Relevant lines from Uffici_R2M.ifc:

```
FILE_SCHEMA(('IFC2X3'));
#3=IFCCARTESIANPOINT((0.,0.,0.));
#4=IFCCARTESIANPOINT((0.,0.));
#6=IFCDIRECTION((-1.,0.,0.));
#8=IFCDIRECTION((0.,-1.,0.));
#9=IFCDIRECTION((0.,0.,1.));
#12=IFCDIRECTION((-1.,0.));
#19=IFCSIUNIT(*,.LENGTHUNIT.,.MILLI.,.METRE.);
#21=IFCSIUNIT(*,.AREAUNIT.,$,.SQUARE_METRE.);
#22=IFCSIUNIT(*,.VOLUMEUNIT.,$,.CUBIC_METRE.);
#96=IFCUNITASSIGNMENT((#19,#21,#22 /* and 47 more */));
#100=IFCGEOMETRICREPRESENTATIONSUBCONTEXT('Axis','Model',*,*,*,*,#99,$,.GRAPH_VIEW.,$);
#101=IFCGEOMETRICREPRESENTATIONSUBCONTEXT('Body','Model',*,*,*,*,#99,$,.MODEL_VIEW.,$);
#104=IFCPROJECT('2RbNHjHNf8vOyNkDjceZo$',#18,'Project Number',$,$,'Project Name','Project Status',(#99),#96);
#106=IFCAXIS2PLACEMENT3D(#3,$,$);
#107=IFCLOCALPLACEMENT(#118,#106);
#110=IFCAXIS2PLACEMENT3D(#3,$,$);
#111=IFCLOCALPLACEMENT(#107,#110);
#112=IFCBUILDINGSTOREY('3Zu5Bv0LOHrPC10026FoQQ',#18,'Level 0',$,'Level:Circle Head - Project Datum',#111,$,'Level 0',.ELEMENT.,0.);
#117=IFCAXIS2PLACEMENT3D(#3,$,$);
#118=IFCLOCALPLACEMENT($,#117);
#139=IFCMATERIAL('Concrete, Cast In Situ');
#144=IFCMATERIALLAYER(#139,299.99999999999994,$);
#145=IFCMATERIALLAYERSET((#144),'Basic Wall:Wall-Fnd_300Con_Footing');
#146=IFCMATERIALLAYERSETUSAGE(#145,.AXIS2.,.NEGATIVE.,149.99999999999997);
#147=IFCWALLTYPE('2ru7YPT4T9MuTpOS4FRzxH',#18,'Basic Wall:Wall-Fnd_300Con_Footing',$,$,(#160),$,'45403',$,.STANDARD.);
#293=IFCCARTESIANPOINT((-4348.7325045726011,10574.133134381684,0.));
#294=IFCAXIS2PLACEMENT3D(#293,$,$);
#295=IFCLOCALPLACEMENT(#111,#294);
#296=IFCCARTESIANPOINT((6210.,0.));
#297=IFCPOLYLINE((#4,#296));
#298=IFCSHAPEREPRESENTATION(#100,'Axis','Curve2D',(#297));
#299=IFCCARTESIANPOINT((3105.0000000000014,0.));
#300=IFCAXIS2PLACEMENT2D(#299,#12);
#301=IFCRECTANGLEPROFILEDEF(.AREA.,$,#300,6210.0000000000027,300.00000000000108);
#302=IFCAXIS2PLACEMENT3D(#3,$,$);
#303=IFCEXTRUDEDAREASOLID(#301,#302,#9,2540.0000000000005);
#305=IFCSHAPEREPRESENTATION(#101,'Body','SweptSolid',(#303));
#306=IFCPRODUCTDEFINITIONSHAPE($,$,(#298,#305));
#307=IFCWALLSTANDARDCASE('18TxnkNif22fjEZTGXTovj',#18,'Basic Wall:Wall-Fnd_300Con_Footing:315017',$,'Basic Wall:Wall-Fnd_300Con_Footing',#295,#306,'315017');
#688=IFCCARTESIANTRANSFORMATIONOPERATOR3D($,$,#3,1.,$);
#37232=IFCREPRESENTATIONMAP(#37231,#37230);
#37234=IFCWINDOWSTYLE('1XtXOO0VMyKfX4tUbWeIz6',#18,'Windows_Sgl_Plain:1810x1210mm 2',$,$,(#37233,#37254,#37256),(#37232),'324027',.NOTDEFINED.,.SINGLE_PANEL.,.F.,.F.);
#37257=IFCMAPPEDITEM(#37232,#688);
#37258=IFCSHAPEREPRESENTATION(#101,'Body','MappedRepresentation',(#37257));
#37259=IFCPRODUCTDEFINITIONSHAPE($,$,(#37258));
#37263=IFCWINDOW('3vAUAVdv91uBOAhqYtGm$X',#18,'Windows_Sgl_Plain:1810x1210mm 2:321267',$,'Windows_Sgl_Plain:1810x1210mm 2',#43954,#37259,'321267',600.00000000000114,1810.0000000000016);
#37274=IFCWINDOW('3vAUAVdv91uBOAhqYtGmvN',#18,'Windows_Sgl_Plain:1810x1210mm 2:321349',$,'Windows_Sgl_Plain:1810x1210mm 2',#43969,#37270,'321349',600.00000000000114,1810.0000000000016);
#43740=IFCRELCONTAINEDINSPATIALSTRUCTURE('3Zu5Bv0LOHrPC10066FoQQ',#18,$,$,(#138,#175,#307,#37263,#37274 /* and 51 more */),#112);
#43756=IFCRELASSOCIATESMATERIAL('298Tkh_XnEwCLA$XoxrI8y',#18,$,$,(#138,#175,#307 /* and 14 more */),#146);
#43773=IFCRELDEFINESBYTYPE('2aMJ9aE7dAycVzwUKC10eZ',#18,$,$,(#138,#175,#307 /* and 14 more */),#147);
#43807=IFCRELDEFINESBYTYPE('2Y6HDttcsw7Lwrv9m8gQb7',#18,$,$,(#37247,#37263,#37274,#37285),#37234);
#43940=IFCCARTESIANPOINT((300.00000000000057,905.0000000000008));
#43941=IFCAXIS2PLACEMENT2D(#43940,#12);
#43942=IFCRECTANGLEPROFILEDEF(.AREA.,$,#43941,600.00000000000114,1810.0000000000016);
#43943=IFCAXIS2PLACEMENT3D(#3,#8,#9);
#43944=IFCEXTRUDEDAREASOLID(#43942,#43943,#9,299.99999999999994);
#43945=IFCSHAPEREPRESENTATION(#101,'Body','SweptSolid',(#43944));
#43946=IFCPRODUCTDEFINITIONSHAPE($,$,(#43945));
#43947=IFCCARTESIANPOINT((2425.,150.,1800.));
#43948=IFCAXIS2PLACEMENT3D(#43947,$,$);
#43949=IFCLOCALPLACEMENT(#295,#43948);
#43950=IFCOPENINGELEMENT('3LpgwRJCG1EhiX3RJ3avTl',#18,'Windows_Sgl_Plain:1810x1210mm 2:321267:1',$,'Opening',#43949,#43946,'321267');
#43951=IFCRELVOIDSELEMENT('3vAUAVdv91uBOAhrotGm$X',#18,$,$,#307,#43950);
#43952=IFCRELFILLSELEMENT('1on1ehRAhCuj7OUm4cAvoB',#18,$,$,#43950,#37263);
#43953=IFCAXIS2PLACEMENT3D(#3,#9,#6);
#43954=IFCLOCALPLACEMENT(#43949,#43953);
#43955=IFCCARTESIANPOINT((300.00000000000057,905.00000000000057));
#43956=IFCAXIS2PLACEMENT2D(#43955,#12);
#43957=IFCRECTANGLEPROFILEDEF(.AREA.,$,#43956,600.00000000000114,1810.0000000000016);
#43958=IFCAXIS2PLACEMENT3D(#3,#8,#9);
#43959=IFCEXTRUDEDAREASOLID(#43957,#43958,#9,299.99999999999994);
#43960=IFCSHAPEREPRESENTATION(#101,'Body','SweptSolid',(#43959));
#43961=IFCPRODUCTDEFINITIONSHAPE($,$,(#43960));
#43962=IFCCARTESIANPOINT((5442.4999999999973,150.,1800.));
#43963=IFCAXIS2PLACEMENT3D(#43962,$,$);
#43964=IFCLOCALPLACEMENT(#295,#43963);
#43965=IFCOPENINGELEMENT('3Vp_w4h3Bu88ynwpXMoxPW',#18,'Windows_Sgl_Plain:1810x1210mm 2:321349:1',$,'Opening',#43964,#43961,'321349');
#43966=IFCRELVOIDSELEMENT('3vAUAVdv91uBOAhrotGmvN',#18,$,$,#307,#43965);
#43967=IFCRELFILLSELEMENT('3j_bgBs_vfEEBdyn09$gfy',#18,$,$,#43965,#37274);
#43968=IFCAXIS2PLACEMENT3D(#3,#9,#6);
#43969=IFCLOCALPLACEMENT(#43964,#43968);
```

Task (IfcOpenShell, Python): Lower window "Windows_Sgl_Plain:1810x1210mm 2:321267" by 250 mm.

```python
import numpy as np
import ifcopenshell
import ifcopenshell.api.geometry
import ifcopenshell.util.placement
import ifcopenshell.util.unit

model = ifcopenshell.open("Uffici_R2M.ifc")
unit_scale = ifcopenshell.util.unit.calculate_unit_scale(model)

window = model.by_guid("3vAUAVdv91uBOAhqYtGm$X")
opening = window.FillsVoids[0].RelatingOpeningElement
dz = -250.0

shift = np.array([0.0, 0.0, dz])
# The window is placed relative to its opening, so it follows when the opening moves.
matrix = ifcopenshell.util.placement.get_local_placement(opening.ObjectPlacement)
matrix[:3, 3] += shift
ifcopenshell.api.geometry.edit_object_placement(
    model, product=opening, matrix=matrix, is_si=False, should_transform_children=True
)

print(f"moved by {dz * unit_scale:+.3f} m")

model.write("Uffici_R2M_edited.ifc")
```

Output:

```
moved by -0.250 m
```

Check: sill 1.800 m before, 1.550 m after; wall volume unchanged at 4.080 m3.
